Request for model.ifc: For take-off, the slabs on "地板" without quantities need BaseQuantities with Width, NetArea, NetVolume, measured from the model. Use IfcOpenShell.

First a look at what the model holds.

```python
import ifcopenshell
import ifcopenshell.util.element
import ifcopenshell.util.unit

model = ifcopenshell.open("model.ifc")
print(model.schema)
for unit_type in ("LENGTHUNIT", "AREAUNIT", "VOLUMEUNIT"):
    print(unit_type, ifcopenshell.util.unit.calculate_unit_scale(model, unit_type))
storey = next(s for s in model.by_type("IfcBuildingStorey") if s.Name == "地板")
slabs = [e for e in ifcopenshell.util.element.get_decomposition(storey) if e.is_a("IfcSlab")]
for e in sorted(slabs, key=lambda e: e.id()):
    print(e.id(), e.is_a(), e.Name, list(ifcopenshell.util.element.get_psets(e, qtos_only=True)), sep=" | ")
```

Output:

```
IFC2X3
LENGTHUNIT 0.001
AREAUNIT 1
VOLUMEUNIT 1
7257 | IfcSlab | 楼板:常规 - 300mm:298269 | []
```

```python
import ifcopenshell
import ifcopenshell.api.pset
import ifcopenshell.geom
import ifcopenshell.util.element
import ifcopenshell.util.shape
import ifcopenshell.util.unit

model = ifcopenshell.open("model.ifc")
unit_scale = ifcopenshell.util.unit.calculate_unit_scale(model)
area_scale = ifcopenshell.util.unit.calculate_unit_scale(model, "AREAUNIT")
volume_scale = ifcopenshell.util.unit.calculate_unit_scale(model, "VOLUMEUNIT")
settings = ifcopenshell.geom.settings()

storey = next(s for s in model.by_type("IfcBuildingStorey") if s.Name == "地板")
slabs = [e for e in ifcopenshell.util.element.get_decomposition(storey) if e.is_a("IfcSlab")]

for e in sorted(slabs, key=lambda e: e.id()):
    if ifcopenshell.util.element.get_psets(e, qtos_only=True, should_inherit=False):
        continue
    # Geometry comes back in metres, in the element's own axes.
    shape = ifcopenshell.geom.create_shape(settings, e)
    values = {
        "Width": ifcopenshell.util.shape.get_z(shape.geometry) / unit_scale,
        "NetArea": ifcopenshell.util.shape.get_footprint_area(shape.geometry) / area_scale,
        "NetVolume": ifcopenshell.util.shape.get_volume(shape.geometry) / volume_scale,
    }
    qto = ifcopenshell.api.pset.add_qto(model, product=e, name="BaseQuantities")
    ifcopenshell.api.pset.edit_qto(model, qto=qto, properties=values)
    print(e.id(), {k: round(v, 3) for k, v in values.items()})

model.write("model-out.ifc")
```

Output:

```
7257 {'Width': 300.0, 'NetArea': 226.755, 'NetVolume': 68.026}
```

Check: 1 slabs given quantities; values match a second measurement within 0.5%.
